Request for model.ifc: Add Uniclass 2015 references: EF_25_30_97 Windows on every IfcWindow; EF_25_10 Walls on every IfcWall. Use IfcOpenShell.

First a look at what the model holds.

```python
import ifcopenshell

model = ifcopenshell.open("model.ifc")
print(model.schema)
print("classifications:", [c.Name for c in model.by_type("IfcClassification")])
for ifc_class in ("IfcDoor", "IfcRoof", "IfcStair", "IfcWall", "IfcWindow"):
    print(ifc_class, len(model.by_type(ifc_class)))
```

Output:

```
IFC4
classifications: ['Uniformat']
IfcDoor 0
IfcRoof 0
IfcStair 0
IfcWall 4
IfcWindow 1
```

```python
import ifcopenshell
import ifcopenshell.api.classification

model = ifcopenshell.open("model.ifc")

system = ifcopenshell.api.classification.add_classification(model, classification="Uniclass 2015")

codes = {
    "IfcWindow": ("EF_25_30_97", "Windows"),
    "IfcWall": ("EF_25_10", "Walls"),
}
for ifc_class, (code, name) in codes.items():
    products = model.by_type(ifc_class)
    ifcopenshell.api.classification.add_reference(
        model, products=products, classification=system, identification=code, name=name
    )
    print(code, len(products))

model.write("model_rev.ifc")
```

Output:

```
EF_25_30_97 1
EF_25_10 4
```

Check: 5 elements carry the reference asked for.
